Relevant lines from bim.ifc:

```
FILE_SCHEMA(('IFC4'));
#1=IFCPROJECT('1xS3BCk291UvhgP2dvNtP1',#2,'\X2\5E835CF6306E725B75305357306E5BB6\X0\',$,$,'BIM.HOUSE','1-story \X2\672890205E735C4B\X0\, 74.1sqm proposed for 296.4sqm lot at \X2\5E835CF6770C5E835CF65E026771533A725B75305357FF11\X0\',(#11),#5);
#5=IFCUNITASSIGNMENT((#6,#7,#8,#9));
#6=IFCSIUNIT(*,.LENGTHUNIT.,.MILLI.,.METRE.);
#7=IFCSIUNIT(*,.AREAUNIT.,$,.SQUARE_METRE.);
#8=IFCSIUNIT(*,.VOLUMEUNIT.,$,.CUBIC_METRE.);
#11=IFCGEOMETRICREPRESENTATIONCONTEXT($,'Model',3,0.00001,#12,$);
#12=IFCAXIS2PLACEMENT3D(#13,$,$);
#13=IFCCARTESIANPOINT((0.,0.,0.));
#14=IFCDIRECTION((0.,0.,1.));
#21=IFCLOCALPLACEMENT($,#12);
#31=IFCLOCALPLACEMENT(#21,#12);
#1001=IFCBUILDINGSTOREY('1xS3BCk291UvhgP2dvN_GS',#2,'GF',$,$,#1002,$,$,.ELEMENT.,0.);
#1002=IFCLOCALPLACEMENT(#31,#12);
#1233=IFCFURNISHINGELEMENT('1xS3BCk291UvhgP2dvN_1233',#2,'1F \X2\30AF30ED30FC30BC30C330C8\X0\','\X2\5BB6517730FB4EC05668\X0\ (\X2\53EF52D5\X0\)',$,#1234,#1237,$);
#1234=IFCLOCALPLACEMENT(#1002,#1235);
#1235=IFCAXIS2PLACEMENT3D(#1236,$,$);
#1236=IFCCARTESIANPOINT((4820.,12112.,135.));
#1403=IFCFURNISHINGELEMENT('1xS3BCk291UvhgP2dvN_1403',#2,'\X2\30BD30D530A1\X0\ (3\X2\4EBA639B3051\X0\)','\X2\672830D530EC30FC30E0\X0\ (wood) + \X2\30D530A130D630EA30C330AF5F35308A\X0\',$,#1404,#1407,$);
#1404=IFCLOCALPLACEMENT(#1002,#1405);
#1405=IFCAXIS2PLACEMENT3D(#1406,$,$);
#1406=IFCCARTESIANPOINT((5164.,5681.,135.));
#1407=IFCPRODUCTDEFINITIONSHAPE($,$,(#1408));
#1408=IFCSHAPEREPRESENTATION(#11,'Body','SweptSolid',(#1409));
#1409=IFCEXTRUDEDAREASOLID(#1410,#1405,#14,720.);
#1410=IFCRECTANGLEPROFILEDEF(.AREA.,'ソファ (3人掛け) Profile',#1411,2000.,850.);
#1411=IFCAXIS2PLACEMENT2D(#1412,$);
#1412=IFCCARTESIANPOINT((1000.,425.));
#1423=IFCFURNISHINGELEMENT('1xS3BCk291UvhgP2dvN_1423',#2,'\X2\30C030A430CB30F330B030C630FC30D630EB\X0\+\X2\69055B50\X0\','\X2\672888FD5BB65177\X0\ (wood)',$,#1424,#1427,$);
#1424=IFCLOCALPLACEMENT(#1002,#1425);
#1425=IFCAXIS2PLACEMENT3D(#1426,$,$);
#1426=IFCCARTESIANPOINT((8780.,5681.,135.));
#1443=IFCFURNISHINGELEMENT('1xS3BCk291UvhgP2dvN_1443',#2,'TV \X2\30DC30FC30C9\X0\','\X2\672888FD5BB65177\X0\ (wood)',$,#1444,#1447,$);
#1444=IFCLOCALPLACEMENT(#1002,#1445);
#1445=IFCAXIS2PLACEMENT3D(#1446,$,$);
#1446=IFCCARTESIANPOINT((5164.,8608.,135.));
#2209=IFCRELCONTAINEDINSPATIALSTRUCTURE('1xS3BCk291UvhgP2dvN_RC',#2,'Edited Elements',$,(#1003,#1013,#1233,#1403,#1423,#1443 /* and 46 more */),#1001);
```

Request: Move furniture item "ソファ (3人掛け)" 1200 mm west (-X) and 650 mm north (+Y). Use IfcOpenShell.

```python
import ifcopenshell
import ifcopenshell.api.geometry
import ifcopenshell.util.placement

model = ifcopenshell.open("bim.ifc")

item = model.by_guid("1xS3BCk291UvhgP2dvN_1403")
matrix = ifcopenshell.util.placement.get_local_placement(item.ObjectPlacement)
matrix[0, 3] -= 1200.0
matrix[1, 3] += 650.0
ifcopenshell.api.geometry.edit_object_placement(model, product=item, matrix=matrix, is_si=False)

print(ifcopenshell.util.placement.get_local_placement(item.ObjectPlacement).round(3) + 0.0)

model.write("bim-out.ifc")
```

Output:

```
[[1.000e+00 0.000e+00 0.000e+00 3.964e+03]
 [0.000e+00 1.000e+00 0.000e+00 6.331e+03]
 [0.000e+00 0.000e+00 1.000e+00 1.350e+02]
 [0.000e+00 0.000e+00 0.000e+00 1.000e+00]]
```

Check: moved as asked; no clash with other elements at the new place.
